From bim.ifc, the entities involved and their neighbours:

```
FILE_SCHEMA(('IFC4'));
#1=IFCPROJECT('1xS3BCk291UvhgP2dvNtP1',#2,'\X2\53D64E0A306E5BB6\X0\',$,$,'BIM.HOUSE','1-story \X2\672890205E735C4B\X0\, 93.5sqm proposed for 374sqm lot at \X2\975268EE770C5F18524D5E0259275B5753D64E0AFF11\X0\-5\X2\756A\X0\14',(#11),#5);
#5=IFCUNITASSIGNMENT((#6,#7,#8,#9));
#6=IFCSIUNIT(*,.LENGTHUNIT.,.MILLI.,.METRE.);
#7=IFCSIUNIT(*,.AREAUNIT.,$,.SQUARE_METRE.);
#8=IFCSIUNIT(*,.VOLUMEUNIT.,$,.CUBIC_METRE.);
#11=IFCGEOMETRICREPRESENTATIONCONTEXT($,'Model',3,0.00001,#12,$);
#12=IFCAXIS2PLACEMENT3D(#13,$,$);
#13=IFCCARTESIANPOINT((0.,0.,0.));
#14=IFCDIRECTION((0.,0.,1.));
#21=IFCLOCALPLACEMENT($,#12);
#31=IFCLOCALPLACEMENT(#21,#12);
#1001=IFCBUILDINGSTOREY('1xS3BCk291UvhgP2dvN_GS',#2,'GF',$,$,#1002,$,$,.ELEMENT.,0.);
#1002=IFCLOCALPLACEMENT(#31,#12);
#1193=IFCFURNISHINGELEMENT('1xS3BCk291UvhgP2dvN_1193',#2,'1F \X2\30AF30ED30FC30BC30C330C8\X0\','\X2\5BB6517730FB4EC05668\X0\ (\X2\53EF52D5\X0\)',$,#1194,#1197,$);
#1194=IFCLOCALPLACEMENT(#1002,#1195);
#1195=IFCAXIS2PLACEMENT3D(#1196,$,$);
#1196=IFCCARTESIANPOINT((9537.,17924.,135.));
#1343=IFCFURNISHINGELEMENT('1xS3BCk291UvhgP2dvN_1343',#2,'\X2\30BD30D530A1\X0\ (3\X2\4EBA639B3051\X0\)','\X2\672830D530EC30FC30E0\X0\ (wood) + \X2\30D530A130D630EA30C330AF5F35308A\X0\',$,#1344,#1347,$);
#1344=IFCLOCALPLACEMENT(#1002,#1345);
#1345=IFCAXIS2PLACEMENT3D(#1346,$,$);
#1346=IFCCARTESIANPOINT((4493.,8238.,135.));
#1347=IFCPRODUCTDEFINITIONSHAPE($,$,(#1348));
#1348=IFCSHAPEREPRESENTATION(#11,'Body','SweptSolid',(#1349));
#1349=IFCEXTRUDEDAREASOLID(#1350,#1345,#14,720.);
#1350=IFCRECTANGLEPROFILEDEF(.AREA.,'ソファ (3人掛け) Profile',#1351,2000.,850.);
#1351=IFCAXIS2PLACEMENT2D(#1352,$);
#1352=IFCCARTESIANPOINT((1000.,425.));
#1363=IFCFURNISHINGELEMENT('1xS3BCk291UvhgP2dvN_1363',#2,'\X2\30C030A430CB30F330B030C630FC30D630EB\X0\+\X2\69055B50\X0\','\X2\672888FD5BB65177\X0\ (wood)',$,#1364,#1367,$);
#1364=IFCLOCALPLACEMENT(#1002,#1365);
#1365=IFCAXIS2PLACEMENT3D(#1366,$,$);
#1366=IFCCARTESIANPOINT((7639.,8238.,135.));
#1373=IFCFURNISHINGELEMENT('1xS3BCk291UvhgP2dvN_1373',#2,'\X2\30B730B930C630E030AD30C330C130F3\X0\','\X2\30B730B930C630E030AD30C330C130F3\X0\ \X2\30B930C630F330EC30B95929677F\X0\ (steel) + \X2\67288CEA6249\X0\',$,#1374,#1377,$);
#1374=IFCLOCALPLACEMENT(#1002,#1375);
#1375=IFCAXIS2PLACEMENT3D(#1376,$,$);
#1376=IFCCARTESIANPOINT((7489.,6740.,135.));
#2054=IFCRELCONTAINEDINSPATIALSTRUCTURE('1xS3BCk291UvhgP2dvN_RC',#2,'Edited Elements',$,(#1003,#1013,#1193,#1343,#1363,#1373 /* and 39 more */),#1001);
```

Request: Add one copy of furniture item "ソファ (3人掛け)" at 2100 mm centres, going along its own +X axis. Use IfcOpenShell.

```python
import ifcopenshell
import ifcopenshell.api.geometry
import ifcopenshell.api.root
import ifcopenshell.util.element
import ifcopenshell.util.placement
import ifcopenshell.util.unit

model = ifcopenshell.open("bim.ifc")
unit_scale = ifcopenshell.util.unit.calculate_unit_scale(model)


def reuse_history(source, copy):
    """copy_class also copies each property set's owner history, people and application; keep the originals."""
    for rel in copy.IsDefinedBy:
        if rel.is_a("IfcRelDefinesByProperties") and (history := rel.RelatingPropertyDefinition.OwnerHistory):
            rel.RelatingPropertyDefinition.OwnerHistory = source.OwnerHistory
            ifcopenshell.util.element.remove_deep2(model, history)


source = model.by_guid("1xS3BCk291UvhgP2dvN_1343")
base = ifcopenshell.util.placement.get_local_placement(source.ObjectPlacement)
step = base[:3, 0] * 2.1 / unit_scale

for i in range(1, 2):
    copy = ifcopenshell.api.root.copy_class(model, product=source)
    copy.Representation = ifcopenshell.util.element.copy_deep(
        model, source.Representation, exclude=["IfcGeometricRepresentationContext", "IfcRepresentationMap"]
    )
    reuse_history(source, copy)
    matrix = base.copy()
    matrix[:3, 3] += i * step
    print("added at", matrix[:3, 3].round(3) + 0.0)
    ifcopenshell.api.geometry.edit_object_placement(model, product=copy, matrix=matrix, is_si=False)

model.write("bim_v2.ifc")
```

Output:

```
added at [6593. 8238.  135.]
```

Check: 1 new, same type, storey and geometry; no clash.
